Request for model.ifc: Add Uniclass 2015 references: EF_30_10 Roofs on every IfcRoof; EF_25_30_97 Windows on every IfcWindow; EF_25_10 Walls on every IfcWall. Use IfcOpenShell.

First a look at what the model holds.

```python
import ifcopenshell

model = ifcopenshell.open("model.ifc")
print(model.schema)
print("classifications:", [c.Name for c in model.by_type("IfcClassification")])
for ifc_class in ("IfcDoor", "IfcRoof", "IfcStair", "IfcWall", "IfcWindow"):
    print(ifc_class, len(model.by_type(ifc_class)))
```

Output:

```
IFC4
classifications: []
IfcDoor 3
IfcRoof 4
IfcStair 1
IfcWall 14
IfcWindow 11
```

```python
import ifcopenshell
import ifcopenshell.api.classification

model = ifcopenshell.open("model.ifc")

system = ifcopenshell.api.classification.add_classification(model, classification="Uniclass 2015")

codes = {
    "IfcRoof": ("EF_30_10", "Roofs"),
    "IfcWindow": ("EF_25_30_97", "Windows"),
    "IfcWall": ("EF_25_10", "Walls"),
}
for ifc_class, (code, name) in codes.items():
    products = model.by_type(ifc_class)
    ifcopenshell.api.classification.add_reference(
        model, products=products, classification=system, identification=code, name=name
    )
    print(code, len(products))

model.write("model_updated.ifc")
```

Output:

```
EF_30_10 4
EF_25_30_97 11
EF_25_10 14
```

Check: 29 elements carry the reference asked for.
